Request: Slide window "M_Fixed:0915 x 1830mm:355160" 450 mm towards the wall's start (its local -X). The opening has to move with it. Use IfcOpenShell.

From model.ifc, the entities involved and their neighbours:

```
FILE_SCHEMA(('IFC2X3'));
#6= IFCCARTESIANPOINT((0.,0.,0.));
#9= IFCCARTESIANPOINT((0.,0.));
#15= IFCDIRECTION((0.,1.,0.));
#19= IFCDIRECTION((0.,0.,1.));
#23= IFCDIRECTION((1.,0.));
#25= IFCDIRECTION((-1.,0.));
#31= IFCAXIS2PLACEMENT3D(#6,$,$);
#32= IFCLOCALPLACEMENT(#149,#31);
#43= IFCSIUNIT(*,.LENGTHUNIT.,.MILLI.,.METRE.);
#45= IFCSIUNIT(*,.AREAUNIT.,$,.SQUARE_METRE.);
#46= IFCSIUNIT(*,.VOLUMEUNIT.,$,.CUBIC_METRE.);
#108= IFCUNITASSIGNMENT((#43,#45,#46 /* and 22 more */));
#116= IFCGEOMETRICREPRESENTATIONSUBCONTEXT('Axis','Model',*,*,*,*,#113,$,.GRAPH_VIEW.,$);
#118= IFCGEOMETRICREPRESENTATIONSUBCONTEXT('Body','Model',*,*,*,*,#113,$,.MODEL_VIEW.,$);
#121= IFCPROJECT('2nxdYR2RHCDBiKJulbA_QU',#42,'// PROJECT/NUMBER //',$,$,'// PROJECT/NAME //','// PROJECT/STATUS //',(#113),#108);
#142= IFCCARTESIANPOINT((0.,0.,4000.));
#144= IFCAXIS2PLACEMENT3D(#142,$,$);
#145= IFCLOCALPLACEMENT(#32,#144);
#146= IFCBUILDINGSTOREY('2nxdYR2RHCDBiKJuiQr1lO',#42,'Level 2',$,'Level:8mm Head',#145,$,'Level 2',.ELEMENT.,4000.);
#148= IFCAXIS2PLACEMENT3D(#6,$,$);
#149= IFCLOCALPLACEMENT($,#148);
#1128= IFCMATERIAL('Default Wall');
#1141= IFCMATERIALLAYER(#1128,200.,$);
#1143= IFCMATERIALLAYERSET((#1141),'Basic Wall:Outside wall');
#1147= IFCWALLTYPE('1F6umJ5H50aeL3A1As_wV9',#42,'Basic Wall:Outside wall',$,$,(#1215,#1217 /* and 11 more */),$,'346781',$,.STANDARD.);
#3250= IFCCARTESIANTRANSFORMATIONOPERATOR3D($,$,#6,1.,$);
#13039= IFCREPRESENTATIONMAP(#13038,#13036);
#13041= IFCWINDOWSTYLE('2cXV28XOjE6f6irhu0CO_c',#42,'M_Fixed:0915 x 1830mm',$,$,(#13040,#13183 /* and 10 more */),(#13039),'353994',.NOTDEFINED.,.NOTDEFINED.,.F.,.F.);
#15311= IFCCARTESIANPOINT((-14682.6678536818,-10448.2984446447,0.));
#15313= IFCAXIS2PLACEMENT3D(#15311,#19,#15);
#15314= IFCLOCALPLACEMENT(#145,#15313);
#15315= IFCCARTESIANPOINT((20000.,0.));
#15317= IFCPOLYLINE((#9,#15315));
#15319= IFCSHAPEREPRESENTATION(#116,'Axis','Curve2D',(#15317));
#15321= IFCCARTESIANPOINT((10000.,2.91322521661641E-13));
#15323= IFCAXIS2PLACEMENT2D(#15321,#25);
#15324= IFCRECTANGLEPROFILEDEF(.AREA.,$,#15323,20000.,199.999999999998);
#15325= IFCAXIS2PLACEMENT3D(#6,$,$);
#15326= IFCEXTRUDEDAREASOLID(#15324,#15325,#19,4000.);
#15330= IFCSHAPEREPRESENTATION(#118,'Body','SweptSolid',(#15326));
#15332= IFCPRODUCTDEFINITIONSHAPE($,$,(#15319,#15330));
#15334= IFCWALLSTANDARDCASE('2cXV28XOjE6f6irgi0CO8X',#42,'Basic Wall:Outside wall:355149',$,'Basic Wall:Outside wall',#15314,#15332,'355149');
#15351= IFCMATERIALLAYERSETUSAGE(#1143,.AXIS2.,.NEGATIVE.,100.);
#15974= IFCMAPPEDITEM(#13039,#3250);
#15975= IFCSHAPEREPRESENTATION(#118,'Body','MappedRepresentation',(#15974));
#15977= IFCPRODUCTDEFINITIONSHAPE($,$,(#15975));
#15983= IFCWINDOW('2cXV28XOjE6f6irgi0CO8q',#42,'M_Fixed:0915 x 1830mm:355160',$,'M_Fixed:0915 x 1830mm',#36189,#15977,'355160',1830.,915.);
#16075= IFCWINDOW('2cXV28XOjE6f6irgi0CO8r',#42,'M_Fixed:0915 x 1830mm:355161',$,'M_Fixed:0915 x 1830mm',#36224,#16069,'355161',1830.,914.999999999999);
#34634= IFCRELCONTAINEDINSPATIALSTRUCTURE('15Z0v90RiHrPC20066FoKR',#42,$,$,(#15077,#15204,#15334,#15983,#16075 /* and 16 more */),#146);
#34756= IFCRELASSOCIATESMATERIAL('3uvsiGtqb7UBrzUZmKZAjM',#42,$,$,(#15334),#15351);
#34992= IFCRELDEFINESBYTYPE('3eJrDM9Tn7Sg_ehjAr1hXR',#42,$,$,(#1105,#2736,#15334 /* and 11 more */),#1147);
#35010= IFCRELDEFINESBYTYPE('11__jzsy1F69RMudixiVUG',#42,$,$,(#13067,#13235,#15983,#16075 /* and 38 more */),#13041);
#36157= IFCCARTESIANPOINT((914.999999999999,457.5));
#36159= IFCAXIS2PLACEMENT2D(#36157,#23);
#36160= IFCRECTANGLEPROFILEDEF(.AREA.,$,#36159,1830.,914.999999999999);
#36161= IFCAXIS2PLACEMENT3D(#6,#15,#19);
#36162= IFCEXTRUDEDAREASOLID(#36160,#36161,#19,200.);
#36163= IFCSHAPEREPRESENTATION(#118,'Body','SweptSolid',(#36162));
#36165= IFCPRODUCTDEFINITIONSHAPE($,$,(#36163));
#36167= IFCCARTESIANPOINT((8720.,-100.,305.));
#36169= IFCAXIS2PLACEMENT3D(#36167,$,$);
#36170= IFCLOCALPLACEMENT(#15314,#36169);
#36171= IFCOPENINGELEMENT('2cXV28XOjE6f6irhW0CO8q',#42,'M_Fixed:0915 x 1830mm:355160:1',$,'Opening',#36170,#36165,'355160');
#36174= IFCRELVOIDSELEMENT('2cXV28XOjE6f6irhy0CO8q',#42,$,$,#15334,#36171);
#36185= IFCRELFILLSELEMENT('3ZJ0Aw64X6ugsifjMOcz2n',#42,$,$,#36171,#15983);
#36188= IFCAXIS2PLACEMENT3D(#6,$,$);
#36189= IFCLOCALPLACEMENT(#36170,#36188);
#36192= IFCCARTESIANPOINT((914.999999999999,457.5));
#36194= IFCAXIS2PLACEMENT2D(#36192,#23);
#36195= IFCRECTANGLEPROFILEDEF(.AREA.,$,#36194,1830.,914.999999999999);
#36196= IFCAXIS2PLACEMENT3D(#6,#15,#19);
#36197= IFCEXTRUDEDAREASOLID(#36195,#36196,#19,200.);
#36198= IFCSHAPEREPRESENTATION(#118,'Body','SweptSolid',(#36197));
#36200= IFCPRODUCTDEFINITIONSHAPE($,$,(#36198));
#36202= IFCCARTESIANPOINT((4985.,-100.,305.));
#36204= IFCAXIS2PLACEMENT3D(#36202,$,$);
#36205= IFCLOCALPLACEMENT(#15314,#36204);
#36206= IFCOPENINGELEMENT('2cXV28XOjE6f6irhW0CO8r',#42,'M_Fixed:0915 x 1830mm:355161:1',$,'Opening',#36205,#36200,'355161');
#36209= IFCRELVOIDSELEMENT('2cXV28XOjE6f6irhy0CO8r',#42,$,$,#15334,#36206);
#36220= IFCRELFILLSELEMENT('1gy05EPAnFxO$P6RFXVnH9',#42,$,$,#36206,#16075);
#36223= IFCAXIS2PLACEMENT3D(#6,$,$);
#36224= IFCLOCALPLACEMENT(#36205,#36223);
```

```python
import ifcopenshell
import ifcopenshell.api.geometry
import ifcopenshell.util.placement
import ifcopenshell.util.unit

model = ifcopenshell.open("model.ifc")
unit_scale = ifcopenshell.util.unit.calculate_unit_scale(model)

window = model.by_guid("2cXV28XOjE6f6irgi0CO8q")
opening = window.FillsVoids[0].RelatingOpeningElement
wall = opening.VoidsElements[0].RelatingBuildingElement

wall_matrix = ifcopenshell.util.placement.get_local_placement(wall.ObjectPlacement)
shift = wall_matrix[:3, 0] * -0.45 / unit_scale
before = ifcopenshell.util.placement.get_local_placement(window.ObjectPlacement)[:3, 3].copy()

# The window is placed relative to its opening, so it follows when the opening moves.
matrix = ifcopenshell.util.placement.get_local_placement(opening.ObjectPlacement)
matrix[:3, 3] += shift
ifcopenshell.api.geometry.edit_object_placement(
    model, product=opening, matrix=matrix, is_si=False, should_transform_children=True
)

after = ifcopenshell.util.placement.get_local_placement(window.ObjectPlacement)[:3, 3]
print("window moved by", (after - before).round(3) + 0.0)

model.write("model_edited.ifc")
```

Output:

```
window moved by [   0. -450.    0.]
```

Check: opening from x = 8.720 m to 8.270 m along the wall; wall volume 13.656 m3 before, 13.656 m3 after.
